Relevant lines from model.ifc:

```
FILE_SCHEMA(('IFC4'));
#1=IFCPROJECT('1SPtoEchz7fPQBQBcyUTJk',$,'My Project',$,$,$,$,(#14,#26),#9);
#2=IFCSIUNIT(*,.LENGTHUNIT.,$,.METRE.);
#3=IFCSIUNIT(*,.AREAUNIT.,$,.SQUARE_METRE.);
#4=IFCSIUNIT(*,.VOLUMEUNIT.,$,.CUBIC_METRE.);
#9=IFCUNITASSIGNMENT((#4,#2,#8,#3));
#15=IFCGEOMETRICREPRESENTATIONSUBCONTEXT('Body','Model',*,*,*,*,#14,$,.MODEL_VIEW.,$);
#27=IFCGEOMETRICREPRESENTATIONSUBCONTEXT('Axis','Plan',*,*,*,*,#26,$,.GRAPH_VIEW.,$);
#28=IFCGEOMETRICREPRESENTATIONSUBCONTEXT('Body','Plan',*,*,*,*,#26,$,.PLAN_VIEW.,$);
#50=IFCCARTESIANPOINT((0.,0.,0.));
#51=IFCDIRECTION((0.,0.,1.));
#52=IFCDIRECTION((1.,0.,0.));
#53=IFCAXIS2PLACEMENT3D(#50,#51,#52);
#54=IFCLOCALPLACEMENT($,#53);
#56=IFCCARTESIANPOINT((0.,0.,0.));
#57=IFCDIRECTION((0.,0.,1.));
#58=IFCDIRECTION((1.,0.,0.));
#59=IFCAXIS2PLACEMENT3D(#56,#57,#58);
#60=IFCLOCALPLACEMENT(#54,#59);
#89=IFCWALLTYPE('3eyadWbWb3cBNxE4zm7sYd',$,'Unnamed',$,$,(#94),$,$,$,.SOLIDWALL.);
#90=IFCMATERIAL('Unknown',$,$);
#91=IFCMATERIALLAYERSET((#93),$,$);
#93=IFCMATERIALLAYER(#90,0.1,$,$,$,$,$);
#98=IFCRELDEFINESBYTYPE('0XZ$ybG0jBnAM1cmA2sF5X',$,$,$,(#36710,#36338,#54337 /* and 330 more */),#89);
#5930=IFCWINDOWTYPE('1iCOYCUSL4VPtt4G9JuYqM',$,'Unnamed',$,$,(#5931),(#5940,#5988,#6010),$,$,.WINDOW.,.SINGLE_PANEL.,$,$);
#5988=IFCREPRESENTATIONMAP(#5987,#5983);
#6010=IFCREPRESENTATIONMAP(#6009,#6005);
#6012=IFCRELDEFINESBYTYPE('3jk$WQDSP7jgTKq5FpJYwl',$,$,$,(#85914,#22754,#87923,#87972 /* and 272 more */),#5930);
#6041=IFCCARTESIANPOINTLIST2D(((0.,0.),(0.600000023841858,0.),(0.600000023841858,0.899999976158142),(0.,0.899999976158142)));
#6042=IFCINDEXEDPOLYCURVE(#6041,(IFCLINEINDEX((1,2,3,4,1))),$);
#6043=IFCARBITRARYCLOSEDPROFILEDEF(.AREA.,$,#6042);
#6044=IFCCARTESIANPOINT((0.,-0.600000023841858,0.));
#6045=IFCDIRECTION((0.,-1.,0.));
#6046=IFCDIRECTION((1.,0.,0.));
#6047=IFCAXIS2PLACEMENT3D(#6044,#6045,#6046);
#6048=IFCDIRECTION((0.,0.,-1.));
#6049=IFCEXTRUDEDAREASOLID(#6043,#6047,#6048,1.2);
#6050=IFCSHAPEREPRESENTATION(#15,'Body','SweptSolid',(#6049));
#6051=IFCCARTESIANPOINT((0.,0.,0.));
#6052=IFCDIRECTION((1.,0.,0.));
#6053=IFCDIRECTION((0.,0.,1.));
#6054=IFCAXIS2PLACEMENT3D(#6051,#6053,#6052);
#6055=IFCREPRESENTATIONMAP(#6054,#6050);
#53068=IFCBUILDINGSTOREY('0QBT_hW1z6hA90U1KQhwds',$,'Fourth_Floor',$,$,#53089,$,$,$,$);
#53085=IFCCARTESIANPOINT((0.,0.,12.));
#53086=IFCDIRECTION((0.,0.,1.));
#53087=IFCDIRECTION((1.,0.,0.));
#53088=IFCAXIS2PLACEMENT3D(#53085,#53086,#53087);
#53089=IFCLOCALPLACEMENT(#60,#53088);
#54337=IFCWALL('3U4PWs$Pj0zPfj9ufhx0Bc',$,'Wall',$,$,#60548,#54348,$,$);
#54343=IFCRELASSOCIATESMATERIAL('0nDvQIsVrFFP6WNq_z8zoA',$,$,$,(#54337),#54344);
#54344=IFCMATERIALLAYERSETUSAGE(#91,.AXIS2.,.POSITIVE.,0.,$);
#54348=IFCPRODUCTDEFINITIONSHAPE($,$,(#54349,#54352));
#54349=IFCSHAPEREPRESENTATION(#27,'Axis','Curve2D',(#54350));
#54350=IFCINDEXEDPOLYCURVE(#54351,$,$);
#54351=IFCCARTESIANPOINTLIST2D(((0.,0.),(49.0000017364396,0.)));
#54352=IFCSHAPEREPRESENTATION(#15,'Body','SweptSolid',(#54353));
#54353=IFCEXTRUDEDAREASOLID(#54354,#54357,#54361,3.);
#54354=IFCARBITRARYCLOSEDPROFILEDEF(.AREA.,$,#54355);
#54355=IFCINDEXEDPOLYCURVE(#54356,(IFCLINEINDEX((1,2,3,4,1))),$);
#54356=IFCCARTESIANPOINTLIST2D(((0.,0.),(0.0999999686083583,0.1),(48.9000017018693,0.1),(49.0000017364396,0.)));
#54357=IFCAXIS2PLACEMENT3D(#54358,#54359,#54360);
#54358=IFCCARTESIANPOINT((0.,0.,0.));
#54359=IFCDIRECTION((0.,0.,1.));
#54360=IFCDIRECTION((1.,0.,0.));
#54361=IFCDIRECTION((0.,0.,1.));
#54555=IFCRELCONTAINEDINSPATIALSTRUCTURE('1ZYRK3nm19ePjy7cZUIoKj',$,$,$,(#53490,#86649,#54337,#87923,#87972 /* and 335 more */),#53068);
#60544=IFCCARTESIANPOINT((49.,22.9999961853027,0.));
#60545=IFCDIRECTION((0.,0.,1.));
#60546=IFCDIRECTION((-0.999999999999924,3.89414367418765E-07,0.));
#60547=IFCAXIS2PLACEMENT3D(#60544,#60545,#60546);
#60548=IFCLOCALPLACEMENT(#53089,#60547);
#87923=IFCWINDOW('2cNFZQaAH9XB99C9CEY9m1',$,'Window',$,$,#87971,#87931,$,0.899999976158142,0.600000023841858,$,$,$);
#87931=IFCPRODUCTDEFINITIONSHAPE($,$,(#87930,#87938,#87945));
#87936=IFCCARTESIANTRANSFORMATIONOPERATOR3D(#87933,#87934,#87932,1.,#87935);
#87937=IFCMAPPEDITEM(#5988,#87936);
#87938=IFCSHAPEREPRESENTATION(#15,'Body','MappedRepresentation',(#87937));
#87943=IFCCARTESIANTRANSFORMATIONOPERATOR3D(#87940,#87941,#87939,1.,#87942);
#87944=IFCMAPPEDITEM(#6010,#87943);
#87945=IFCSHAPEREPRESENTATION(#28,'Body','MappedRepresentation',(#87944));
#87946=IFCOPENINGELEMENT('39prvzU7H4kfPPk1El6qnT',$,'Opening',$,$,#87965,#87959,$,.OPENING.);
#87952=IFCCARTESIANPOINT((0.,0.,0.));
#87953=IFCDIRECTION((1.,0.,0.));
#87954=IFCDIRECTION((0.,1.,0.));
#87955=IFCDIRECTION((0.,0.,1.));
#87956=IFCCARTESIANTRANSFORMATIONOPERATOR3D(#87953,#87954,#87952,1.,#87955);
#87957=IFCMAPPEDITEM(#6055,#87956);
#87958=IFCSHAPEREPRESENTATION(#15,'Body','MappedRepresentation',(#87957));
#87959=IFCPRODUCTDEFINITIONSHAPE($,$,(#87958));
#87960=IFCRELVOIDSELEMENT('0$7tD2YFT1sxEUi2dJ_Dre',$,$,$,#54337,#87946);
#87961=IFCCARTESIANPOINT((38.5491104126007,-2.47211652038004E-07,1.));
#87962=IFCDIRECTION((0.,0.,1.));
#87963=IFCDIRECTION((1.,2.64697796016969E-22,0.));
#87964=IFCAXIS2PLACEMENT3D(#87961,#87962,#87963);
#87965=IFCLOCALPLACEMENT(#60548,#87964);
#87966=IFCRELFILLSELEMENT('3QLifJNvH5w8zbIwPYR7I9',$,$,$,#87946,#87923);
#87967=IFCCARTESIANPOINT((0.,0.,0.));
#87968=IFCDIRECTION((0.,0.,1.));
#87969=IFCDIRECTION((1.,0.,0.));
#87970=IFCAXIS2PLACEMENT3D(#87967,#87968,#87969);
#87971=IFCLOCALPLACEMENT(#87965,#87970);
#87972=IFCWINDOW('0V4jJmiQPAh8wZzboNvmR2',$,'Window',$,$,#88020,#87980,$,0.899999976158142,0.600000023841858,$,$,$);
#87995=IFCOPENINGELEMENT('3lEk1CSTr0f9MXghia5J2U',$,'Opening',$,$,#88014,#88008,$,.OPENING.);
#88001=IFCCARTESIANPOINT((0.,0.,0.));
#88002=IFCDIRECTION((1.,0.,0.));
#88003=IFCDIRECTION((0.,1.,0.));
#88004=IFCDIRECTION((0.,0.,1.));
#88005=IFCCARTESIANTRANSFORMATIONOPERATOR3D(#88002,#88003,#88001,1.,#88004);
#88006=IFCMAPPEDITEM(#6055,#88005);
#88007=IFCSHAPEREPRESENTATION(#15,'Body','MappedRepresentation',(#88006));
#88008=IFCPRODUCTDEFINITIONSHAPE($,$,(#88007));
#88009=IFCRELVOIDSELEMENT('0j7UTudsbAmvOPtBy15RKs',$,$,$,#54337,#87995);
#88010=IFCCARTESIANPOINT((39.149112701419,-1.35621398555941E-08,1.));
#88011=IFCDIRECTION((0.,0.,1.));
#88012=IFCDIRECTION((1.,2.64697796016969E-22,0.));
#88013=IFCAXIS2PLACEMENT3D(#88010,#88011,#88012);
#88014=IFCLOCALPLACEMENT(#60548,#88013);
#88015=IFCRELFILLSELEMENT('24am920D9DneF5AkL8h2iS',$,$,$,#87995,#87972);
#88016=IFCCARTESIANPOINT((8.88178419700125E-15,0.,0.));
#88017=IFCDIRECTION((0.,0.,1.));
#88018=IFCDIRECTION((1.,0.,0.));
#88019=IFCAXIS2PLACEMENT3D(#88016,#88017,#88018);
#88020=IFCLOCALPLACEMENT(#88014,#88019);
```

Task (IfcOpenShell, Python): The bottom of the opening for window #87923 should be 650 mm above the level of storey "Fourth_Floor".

```python
import numpy as np
import ifcopenshell
import ifcopenshell.api.geometry
import ifcopenshell.geom
import ifcopenshell.util.element
import ifcopenshell.util.placement
import ifcopenshell.util.shape
import ifcopenshell.util.unit

model = ifcopenshell.open("model.ifc")
unit_scale = ifcopenshell.util.unit.calculate_unit_scale(model)

window = model.by_guid("2cNFZQaAH9XB99C9CEY9m1")
opening = window.FillsVoids[0].RelatingOpeningElement
storey = ifcopenshell.util.element.get_container(window, ifc_class="IfcBuildingStorey")
level = ifcopenshell.util.placement.get_local_placement(storey.ObjectPlacement)[2, 3]

# The opening's origin need not be at the sill, so measure its lowest point.
shape = ifcopenshell.geom.create_shape(ifcopenshell.geom.settings(), opening)
bottom = ifcopenshell.util.shape.get_shape_bottom_elevation(shape, shape.geometry) / unit_scale
dz = level + 0.65 / unit_scale - bottom

shift = np.array([0.0, 0.0, dz])
# The window is placed relative to its opening, so it follows when the opening moves.
matrix = ifcopenshell.util.placement.get_local_placement(opening.ObjectPlacement)
matrix[:3, 3] += shift
ifcopenshell.api.geometry.edit_object_placement(
    model, product=opening, matrix=matrix, is_si=False, should_transform_children=True
)

print(f"moved by {dz * unit_scale:+.3f} m")

model.write("model_updated.ifc")
```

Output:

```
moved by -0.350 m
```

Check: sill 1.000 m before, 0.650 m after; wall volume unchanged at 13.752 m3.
